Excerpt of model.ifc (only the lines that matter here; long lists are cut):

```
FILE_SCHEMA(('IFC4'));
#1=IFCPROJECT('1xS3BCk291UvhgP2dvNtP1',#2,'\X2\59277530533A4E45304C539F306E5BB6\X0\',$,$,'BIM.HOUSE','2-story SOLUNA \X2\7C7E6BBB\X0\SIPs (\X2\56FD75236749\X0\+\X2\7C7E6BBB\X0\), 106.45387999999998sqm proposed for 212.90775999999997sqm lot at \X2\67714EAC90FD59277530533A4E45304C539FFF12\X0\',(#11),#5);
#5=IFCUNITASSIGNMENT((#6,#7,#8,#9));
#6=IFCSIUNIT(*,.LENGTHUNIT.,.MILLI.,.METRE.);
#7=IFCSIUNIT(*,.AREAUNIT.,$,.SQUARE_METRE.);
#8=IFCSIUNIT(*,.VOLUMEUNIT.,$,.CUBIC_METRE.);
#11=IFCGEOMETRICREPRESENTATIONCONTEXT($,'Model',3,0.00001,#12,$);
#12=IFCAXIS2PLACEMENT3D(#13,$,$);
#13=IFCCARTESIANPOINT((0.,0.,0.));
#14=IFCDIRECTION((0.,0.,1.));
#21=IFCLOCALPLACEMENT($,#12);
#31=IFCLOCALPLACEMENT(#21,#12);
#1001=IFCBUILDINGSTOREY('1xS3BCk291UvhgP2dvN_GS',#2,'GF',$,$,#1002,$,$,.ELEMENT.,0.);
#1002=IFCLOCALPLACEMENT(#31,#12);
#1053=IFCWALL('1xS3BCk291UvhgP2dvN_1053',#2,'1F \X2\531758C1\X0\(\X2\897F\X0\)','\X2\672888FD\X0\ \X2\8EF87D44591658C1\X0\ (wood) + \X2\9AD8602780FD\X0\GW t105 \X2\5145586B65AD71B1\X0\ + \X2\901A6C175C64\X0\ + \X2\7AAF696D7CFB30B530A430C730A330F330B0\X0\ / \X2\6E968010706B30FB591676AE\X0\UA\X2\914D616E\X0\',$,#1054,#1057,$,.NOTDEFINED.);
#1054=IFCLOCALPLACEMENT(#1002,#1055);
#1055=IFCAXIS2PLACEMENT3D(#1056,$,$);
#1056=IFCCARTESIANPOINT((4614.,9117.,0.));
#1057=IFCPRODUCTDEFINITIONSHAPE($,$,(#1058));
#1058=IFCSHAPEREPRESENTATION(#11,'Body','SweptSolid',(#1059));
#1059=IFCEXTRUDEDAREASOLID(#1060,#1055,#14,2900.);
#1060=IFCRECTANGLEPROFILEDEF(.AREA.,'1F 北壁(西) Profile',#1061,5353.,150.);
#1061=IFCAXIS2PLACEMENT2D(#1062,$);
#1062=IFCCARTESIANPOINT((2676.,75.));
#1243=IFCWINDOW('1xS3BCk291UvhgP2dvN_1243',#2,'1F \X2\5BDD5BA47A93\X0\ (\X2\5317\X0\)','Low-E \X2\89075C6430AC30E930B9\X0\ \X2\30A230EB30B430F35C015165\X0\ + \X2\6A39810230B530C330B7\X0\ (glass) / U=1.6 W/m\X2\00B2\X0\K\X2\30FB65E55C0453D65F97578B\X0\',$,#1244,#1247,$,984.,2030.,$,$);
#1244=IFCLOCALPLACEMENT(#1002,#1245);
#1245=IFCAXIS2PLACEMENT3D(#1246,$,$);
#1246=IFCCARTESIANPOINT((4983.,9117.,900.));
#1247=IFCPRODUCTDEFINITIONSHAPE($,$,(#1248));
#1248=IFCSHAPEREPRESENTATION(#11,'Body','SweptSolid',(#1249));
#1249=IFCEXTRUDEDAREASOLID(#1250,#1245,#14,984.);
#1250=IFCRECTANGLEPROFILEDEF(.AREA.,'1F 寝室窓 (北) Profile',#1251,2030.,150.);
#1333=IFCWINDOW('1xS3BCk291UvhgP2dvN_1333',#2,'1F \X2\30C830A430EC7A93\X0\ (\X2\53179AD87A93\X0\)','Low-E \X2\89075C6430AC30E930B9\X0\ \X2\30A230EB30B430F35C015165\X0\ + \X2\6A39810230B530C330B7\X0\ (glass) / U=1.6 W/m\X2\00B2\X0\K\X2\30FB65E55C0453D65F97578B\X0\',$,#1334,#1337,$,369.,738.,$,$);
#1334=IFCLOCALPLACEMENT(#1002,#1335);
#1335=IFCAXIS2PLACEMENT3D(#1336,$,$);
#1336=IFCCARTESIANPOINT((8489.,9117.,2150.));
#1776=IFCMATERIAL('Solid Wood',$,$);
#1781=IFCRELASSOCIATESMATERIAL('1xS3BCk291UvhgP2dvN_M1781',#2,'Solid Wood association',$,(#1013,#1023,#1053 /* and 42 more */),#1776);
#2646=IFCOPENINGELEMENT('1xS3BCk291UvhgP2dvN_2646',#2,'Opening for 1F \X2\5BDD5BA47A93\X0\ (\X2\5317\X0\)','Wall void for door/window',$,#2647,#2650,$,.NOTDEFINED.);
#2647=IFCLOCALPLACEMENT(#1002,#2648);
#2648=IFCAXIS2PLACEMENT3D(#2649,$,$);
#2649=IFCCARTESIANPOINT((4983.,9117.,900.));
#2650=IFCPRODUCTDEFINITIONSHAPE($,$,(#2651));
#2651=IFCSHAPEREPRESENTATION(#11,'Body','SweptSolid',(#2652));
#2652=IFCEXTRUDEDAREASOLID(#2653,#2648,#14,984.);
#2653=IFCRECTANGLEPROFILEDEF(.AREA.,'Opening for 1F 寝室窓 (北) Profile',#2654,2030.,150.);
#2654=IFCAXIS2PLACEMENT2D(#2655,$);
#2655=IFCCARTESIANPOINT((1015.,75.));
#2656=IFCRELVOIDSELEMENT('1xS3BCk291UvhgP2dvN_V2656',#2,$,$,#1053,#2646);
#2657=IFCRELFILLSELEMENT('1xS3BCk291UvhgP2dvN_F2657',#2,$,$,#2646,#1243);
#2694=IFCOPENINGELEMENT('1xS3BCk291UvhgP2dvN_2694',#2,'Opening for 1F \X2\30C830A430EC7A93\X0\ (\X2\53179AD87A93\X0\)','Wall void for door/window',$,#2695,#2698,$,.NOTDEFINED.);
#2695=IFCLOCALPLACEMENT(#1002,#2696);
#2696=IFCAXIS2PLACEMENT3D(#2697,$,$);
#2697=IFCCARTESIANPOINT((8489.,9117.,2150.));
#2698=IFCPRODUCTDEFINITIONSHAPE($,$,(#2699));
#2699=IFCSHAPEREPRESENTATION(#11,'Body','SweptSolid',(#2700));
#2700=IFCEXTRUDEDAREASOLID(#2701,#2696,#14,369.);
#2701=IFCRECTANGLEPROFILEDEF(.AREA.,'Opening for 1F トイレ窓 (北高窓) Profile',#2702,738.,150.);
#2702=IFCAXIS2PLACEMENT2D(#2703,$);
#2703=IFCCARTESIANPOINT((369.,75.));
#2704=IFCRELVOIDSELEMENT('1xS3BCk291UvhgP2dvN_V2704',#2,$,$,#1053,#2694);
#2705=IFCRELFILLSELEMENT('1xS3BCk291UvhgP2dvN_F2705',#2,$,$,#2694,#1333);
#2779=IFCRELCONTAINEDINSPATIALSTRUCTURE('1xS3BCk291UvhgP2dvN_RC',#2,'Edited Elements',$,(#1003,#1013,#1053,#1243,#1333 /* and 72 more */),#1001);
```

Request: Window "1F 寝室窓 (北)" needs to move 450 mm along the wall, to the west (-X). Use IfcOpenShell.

```python
import ifcopenshell
import ifcopenshell.api.geometry
import ifcopenshell.util.placement
import ifcopenshell.util.unit

model = ifcopenshell.open("model.ifc")
unit_scale = ifcopenshell.util.unit.calculate_unit_scale(model)

window = model.by_guid("1xS3BCk291UvhgP2dvN_1243")
opening = window.FillsVoids[0].RelatingOpeningElement
wall = opening.VoidsElements[0].RelatingBuildingElement

wall_matrix = ifcopenshell.util.placement.get_local_placement(wall.ObjectPlacement)
shift = wall_matrix[:3, 0] * -0.45 / unit_scale
before = ifcopenshell.util.placement.get_local_placement(window.ObjectPlacement)[:3, 3].copy()

# The window is not placed relative to its opening, so move both.
for product in (opening, window):
    matrix = ifcopenshell.util.placement.get_local_placement(product.ObjectPlacement)
    matrix[:3, 3] += shift
    ifcopenshell.api.geometry.edit_object_placement(model, product=product, matrix=matrix, is_si=False)

after = ifcopenshell.util.placement.get_local_placement(window.ObjectPlacement)[:3, 3]
print("window moved by", (after - before).round(3) + 0.0)

model.write("model-out.ifc")
```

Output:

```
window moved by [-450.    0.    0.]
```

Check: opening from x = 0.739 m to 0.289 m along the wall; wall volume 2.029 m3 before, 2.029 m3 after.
